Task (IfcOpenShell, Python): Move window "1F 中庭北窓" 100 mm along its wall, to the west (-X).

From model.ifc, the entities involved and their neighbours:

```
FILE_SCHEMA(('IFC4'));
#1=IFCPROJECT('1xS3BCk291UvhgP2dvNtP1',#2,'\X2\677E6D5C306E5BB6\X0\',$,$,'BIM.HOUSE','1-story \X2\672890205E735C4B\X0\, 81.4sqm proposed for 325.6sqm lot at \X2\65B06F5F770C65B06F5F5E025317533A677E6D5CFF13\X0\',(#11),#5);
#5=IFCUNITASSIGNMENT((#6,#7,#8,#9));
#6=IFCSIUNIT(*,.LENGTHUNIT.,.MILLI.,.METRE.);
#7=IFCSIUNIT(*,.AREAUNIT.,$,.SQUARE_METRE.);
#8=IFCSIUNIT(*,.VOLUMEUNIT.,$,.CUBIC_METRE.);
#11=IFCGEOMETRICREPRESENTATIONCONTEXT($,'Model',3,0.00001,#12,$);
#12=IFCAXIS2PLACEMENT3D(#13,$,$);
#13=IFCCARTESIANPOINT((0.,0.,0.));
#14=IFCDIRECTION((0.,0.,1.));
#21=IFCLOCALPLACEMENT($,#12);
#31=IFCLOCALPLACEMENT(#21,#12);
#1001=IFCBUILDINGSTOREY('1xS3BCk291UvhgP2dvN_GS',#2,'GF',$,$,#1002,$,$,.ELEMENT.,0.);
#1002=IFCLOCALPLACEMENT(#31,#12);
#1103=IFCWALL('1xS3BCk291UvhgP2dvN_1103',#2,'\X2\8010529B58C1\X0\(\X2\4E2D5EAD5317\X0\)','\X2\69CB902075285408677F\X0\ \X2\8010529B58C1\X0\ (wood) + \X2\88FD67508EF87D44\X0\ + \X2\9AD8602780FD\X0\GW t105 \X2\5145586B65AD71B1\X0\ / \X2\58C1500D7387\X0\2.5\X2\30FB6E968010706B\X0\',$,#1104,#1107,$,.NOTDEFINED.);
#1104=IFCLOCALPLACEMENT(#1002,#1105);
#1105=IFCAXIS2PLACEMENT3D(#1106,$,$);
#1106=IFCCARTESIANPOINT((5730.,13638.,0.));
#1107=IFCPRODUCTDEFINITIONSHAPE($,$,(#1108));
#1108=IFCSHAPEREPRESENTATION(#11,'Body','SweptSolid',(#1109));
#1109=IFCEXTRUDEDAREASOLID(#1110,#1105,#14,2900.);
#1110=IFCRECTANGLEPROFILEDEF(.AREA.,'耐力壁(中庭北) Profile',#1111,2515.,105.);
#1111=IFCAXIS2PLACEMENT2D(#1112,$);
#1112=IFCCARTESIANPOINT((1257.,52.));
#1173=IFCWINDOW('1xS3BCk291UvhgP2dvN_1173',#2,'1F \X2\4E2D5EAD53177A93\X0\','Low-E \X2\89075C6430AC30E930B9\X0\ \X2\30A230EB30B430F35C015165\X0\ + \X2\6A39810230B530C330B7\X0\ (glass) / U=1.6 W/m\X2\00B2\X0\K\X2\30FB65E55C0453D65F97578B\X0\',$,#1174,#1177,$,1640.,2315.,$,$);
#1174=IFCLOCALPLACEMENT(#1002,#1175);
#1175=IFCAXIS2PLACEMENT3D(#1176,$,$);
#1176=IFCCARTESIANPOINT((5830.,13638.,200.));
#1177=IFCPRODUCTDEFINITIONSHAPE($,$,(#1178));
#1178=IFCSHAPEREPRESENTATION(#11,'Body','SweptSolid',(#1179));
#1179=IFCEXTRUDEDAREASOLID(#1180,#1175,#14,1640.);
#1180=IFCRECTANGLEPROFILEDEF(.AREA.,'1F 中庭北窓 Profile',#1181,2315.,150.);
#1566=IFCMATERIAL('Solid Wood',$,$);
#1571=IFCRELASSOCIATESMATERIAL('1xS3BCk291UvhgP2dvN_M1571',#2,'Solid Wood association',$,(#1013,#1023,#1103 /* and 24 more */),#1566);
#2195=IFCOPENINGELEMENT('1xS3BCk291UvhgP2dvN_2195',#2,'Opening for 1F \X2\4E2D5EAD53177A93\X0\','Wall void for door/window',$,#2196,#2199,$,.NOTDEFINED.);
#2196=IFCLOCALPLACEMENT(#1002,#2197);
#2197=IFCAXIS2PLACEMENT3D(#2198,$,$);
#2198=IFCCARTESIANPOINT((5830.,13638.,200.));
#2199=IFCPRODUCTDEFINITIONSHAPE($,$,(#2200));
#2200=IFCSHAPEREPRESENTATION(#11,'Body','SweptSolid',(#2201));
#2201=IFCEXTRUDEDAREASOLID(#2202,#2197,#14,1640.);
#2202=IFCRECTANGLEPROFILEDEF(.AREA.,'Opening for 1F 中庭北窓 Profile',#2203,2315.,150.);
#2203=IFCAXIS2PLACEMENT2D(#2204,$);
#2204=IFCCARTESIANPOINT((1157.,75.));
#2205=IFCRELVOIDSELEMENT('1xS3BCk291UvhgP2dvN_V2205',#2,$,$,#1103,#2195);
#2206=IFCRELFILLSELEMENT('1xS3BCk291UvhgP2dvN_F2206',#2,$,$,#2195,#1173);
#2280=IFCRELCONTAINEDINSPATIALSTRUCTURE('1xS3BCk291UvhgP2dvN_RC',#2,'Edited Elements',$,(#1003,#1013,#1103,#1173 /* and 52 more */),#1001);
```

```python
import ifcopenshell
import ifcopenshell.api.geometry
import ifcopenshell.util.placement
import ifcopenshell.util.unit

model = ifcopenshell.open("model.ifc")
unit_scale = ifcopenshell.util.unit.calculate_unit_scale(model)

window = model.by_guid("1xS3BCk291UvhgP2dvN_1173")
opening = window.FillsVoids[0].RelatingOpeningElement
wall = opening.VoidsElements[0].RelatingBuildingElement

wall_matrix = ifcopenshell.util.placement.get_local_placement(wall.ObjectPlacement)
shift = wall_matrix[:3, 0] * -0.1 / unit_scale
before = ifcopenshell.util.placement.get_local_placement(window.ObjectPlacement)[:3, 3].copy()

# The window is not placed relative to its opening, so move both.
for product in (opening, window):
    matrix = ifcopenshell.util.placement.get_local_placement(product.ObjectPlacement)
    matrix[:3, 3] += shift
    ifcopenshell.api.geometry.edit_object_placement(model, product=product, matrix=matrix, is_si=False)

after = ifcopenshell.util.placement.get_local_placement(window.ObjectPlacement)[:3, 3]
print("window moved by", (after - before).round(3) + 0.0)

model.write("model_edited.ifc")
```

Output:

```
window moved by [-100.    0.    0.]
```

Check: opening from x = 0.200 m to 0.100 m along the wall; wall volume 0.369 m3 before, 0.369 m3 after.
